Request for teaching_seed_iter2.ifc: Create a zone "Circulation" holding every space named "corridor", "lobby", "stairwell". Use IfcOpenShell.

First a look at what the model holds.

```python
import ifcopenshell

model = ifcopenshell.open("teaching_seed_iter2.ifc")
print(model.schema)
seen = {}
for space in model.by_type("IfcSpace"):
    seen[space.LongName] = seen.get(space.LongName, 0) + 1
for name, count in sorted(seen.items(), key=str):
    print(count, "x", name)
print("zones:", [z.Name for z in model.by_type("IfcZone")][:20])
```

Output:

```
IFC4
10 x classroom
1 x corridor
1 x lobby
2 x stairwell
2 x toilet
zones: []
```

```python
import ifcopenshell
import ifcopenshell.api.group
import ifcopenshell.api.root

model = ifcopenshell.open("teaching_seed_iter2.ifc")

names = {"corridor", "lobby", "stairwell"}
spaces = [s for s in model.by_type("IfcSpace") if s.LongName in names]

zone = ifcopenshell.api.root.create_entity(model, ifc_class="IfcZone", name="Circulation")
ifcopenshell.api.group.assign_group(model, products=spaces, group=zone)
print(len(spaces), "spaces in", zone.Name)

model.write("teaching_seed_iter2_rev.ifc")
```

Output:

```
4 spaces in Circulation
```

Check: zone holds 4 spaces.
